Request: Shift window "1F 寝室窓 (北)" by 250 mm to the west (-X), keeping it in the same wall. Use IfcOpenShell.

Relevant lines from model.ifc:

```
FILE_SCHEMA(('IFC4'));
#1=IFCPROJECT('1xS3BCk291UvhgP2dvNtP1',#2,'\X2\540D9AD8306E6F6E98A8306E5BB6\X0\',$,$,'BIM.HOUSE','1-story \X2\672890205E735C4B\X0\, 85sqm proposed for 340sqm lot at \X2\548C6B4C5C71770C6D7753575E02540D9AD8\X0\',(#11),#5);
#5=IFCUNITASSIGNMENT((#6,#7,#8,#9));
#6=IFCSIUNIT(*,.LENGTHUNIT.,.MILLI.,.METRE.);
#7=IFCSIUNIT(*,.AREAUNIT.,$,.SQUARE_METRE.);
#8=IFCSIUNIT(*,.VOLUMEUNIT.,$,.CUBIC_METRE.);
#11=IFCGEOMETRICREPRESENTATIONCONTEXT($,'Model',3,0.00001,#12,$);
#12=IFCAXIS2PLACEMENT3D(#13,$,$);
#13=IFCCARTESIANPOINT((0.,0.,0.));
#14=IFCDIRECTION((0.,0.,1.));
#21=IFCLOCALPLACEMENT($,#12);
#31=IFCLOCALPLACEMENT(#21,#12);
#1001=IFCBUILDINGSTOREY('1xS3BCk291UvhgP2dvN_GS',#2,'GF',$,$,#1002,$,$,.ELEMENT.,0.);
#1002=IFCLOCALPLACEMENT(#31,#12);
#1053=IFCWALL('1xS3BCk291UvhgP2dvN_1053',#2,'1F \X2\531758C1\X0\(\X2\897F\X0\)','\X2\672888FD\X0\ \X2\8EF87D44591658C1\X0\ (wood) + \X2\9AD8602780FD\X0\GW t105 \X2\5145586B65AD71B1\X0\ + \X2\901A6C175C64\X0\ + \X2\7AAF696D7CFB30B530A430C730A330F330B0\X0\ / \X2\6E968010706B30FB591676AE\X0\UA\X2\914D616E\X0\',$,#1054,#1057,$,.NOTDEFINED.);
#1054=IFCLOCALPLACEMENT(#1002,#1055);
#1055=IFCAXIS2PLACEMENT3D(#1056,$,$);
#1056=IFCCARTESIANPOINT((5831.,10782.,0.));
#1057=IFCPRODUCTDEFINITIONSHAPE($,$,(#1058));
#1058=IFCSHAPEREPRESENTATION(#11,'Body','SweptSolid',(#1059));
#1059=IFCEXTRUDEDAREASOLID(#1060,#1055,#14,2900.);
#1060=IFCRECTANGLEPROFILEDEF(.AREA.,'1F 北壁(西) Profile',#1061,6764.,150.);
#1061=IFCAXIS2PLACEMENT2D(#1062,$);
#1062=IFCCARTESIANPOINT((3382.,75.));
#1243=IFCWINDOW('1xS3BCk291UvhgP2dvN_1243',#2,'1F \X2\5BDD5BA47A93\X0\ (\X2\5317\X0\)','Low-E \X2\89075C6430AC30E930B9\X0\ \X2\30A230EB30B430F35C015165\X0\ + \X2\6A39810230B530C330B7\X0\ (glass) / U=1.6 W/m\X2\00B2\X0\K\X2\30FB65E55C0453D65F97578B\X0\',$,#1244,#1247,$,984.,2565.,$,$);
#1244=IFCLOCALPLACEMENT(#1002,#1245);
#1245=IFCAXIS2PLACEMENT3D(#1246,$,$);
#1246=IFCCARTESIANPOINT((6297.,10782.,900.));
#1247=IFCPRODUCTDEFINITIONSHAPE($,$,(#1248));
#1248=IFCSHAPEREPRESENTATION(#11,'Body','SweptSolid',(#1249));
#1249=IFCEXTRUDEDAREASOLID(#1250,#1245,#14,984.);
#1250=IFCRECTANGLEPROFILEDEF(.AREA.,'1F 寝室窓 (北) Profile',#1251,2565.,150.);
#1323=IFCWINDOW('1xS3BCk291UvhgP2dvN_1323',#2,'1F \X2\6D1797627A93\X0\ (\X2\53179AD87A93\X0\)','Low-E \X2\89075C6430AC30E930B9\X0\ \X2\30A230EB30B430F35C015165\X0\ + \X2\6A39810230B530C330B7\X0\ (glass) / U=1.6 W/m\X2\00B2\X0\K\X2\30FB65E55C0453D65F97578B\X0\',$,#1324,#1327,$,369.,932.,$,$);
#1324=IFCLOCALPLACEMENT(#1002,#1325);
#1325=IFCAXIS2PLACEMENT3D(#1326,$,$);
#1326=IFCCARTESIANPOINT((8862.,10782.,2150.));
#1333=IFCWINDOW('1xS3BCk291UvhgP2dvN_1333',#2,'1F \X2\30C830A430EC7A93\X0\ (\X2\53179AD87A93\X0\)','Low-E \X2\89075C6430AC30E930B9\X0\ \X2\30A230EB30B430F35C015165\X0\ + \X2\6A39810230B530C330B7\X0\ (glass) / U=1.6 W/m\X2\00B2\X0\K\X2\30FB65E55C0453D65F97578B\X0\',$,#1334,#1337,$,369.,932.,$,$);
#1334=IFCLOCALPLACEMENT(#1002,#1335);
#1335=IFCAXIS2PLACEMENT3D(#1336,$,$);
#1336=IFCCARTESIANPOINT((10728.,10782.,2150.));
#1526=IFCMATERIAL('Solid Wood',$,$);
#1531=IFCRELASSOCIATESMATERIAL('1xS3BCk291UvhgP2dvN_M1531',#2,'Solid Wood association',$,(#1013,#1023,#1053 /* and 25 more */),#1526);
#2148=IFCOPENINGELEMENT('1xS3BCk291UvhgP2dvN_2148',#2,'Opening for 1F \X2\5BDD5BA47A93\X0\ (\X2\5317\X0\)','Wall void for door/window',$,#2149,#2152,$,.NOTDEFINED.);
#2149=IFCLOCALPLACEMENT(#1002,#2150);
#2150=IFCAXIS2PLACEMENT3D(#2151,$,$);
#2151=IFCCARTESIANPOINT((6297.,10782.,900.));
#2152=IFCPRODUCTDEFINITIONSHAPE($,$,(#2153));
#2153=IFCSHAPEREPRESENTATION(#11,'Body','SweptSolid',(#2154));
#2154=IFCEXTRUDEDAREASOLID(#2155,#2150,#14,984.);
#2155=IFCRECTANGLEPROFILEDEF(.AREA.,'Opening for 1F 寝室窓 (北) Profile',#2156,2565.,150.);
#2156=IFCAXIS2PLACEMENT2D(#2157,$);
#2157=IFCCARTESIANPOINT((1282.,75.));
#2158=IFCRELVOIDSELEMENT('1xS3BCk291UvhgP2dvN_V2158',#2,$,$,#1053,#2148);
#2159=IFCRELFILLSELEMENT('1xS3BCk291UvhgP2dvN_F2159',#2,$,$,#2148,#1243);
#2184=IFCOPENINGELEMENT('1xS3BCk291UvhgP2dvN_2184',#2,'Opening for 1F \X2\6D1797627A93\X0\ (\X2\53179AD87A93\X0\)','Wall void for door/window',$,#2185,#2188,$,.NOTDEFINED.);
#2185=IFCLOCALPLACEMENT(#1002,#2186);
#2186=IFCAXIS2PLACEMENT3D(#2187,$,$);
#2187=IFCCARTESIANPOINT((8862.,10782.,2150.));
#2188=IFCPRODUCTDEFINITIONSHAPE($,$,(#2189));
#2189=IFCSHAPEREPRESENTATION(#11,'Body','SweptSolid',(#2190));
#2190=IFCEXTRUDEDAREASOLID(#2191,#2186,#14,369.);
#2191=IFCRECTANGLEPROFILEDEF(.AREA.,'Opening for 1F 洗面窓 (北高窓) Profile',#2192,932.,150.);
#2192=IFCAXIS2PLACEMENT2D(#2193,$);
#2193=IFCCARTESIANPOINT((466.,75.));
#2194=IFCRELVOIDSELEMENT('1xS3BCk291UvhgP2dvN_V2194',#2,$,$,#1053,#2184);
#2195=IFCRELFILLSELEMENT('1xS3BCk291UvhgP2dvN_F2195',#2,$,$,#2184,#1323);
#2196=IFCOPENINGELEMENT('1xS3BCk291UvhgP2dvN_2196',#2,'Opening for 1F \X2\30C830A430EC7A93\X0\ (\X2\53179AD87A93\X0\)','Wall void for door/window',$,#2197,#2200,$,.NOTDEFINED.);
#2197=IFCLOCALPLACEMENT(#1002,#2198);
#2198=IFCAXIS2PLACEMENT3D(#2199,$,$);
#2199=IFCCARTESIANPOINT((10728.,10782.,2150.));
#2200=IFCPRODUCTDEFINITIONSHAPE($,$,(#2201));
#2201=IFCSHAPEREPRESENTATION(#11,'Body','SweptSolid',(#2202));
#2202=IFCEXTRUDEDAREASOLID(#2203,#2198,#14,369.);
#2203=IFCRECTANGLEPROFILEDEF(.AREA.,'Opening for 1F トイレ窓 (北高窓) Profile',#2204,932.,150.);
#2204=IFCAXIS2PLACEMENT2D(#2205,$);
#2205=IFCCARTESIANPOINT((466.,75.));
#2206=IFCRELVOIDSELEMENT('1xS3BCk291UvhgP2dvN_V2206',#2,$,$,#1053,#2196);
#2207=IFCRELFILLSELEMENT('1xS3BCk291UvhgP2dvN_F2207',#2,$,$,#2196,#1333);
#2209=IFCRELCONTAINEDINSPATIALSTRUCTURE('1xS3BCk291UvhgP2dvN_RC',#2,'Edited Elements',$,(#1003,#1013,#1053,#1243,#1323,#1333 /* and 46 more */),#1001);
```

```python
import ifcopenshell
import ifcopenshell.api.geometry
import ifcopenshell.util.placement

model = ifcopenshell.open("model.ifc")

window = model.by_id(1243)
opening = window.FillsVoids[0].RelatingOpeningElement
wall = opening.VoidsElements[0].RelatingBuildingElement

wall_matrix = ifcopenshell.util.placement.get_local_placement(wall.ObjectPlacement)
shift = wall_matrix[:3, 0] * -250.0
before = ifcopenshell.util.placement.get_local_placement(window.ObjectPlacement)[:3, 3].copy()

# The window is not placed relative to its opening, so move both.
for product in (opening, window):
    matrix = ifcopenshell.util.placement.get_local_placement(product.ObjectPlacement)
    matrix[:3, 3] += shift
    ifcopenshell.api.geometry.edit_object_placement(model, product=product, matrix=matrix, is_si=False)

after = ifcopenshell.util.placement.get_local_placement(window.ObjectPlacement)[:3, 3]
print("window moved by", (after - before).round(3) + 0.0)

model.write("model_edited.ifc")
```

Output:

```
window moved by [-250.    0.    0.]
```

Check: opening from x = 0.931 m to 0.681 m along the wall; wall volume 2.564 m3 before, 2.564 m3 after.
